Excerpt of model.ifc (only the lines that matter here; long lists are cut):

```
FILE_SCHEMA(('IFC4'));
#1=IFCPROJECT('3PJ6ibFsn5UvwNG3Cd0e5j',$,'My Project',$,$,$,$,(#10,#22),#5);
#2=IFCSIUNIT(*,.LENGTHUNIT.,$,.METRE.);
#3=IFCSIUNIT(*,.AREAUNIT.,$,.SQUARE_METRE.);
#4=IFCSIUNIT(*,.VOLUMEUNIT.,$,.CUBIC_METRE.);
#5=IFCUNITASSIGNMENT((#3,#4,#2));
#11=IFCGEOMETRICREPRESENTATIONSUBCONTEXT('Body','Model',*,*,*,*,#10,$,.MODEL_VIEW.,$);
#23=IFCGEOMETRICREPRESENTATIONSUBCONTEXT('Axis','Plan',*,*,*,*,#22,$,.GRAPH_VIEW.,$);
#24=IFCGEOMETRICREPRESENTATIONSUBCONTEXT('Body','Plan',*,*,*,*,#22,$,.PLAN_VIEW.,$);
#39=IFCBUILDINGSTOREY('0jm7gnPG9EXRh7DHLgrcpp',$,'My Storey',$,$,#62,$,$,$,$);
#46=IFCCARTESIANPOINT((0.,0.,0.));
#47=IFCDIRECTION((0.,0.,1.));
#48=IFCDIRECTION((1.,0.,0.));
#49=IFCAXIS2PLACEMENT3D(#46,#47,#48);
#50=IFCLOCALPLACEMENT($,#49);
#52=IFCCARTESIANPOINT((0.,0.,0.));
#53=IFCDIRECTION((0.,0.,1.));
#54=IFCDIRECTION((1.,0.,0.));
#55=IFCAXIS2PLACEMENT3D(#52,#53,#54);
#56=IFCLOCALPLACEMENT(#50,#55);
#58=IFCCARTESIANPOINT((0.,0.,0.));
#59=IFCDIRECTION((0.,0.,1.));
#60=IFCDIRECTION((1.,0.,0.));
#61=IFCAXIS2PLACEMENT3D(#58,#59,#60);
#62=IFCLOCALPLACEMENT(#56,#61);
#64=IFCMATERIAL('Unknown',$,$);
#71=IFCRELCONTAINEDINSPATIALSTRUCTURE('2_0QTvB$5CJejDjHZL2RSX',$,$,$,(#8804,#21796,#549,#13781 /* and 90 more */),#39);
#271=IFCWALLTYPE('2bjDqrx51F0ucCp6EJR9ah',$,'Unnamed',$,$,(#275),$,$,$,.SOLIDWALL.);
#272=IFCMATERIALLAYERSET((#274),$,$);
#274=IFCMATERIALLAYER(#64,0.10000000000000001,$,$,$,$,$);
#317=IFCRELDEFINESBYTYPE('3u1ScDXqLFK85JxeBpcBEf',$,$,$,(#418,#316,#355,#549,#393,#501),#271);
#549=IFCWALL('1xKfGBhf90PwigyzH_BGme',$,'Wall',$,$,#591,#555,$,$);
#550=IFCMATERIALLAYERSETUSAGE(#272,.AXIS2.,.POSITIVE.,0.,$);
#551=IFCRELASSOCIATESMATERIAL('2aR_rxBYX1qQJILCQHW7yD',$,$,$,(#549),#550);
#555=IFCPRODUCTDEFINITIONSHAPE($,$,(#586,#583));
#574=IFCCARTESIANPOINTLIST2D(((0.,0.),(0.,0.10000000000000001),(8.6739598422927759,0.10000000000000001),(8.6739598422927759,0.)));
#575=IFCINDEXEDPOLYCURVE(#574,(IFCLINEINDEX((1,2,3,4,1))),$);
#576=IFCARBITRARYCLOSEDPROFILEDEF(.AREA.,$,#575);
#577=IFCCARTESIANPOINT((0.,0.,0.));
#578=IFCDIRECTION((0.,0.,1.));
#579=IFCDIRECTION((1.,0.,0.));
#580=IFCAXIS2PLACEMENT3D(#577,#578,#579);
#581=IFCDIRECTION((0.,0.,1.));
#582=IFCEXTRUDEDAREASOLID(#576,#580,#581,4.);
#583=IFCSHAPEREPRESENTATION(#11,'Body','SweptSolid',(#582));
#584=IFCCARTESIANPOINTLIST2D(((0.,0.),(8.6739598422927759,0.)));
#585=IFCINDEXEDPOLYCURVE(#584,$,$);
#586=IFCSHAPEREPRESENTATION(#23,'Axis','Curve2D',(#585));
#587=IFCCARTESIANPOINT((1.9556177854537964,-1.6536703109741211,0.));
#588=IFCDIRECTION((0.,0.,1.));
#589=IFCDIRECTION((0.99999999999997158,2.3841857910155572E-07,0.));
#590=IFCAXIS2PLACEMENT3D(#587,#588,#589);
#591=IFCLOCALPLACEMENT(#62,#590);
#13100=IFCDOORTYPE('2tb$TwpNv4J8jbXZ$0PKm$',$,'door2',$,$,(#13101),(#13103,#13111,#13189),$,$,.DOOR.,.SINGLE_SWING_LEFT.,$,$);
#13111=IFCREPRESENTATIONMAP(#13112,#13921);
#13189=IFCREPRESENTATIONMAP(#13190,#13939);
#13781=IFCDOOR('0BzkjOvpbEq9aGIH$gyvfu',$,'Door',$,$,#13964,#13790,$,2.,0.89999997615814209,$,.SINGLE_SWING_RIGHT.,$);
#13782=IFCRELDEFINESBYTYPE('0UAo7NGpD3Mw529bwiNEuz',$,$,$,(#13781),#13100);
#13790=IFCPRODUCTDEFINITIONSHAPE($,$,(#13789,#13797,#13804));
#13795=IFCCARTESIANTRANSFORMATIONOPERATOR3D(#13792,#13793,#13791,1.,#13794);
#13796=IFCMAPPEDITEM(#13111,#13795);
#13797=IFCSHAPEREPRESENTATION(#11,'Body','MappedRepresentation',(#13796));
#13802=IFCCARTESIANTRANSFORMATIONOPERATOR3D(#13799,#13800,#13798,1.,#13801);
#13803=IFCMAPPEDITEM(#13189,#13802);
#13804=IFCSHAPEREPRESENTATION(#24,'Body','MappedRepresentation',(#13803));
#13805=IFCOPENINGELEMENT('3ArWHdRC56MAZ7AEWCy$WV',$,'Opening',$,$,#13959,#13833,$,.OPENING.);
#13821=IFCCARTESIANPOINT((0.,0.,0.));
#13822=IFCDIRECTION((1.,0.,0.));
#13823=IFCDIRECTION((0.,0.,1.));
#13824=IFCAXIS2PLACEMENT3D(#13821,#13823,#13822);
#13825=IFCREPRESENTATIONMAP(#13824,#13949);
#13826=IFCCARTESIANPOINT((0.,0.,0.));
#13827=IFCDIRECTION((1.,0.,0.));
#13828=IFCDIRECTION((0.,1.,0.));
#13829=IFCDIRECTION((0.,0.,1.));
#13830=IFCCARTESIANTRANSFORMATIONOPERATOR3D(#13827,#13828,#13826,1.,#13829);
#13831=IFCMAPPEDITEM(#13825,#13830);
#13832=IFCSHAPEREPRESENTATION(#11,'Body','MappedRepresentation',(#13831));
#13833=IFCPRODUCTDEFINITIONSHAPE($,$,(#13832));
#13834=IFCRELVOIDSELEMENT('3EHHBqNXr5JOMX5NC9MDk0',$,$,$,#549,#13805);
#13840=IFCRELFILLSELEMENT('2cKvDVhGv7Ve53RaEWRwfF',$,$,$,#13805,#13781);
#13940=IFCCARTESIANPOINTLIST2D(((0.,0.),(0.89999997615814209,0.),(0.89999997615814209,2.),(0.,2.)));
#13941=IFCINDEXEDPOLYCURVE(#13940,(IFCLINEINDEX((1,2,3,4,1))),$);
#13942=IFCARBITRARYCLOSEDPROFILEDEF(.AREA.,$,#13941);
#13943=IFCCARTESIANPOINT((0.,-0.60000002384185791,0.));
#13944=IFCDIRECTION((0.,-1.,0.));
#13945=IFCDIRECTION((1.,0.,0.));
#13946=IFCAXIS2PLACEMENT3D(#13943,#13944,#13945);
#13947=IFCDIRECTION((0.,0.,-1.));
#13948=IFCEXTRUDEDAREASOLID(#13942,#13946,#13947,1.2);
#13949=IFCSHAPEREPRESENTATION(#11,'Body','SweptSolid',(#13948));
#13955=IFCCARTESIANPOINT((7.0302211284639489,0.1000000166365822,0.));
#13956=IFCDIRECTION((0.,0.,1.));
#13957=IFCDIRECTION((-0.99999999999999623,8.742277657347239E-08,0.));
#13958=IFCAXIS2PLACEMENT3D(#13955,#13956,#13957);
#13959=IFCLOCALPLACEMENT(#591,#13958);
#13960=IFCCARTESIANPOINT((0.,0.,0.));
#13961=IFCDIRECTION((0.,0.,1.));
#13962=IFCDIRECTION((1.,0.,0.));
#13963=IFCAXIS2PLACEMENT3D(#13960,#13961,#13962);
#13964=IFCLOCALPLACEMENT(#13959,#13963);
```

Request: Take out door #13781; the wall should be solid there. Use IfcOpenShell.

```python
import ifcopenshell
import ifcopenshell.api.feature
import ifcopenshell.api.root
import ifcopenshell.geom
import ifcopenshell.util.shape

model = ifcopenshell.open("model.ifc")
settings = ifcopenshell.geom.settings()


def volume(element):
    """Net volume in cubic metres, openings subtracted."""
    shape = ifcopenshell.geom.create_shape(settings, element)
    return ifcopenshell.util.shape.get_volume(shape.geometry)


door = model.by_guid("0BzkjOvpbEq9aGIH$gyvfu")
opening = door.FillsVoids[0].RelatingOpeningElement
wall = opening.VoidsElements[0].RelatingBuildingElement
before = volume(wall)

ifcopenshell.api.root.remove_product(model, product=door)
ifcopenshell.api.feature.remove_feature(model, feature=opening)

after = volume(wall)

print(f"wall volume {before:.3f} -> {after:.3f} m3")

model.write("model_rev.ifc")
```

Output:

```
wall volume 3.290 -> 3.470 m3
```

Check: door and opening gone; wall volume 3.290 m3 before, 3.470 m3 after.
